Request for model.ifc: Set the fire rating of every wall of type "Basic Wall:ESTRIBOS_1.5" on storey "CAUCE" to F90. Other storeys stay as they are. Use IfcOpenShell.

First a look at what the model holds.

```python
import ifcopenshell
import ifcopenshell.util.element

model = ifcopenshell.open("model.ifc")
print(model.schema)
storey = next(s for s in model.by_type("IfcBuildingStorey") if s.Name == "CAUCE")
walls = [e for e in ifcopenshell.util.element.get_decomposition(storey) if e.is_a("IfcWall")]
seen = {}
for e in walls:
    element_type = ifcopenshell.util.element.get_type(e)
    key = (element_type.Name if element_type != e and element_type else None, ifcopenshell.util.element.get_pset(e, "Pset_WallCommon", "FireRating"))
    seen[key] = seen.get(key, 0) + 1
for (name, value), count in sorted(seen.items(), key=str):
    print(count, "x", name, "|", value)
```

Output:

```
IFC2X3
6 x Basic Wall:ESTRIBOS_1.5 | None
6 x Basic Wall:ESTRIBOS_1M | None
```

```python
import ifcopenshell
import ifcopenshell.api.pset
import ifcopenshell.util.element

model = ifcopenshell.open("model.ifc")

storey = next(s for s in model.by_type("IfcBuildingStorey") if s.Name == "CAUCE")
walls = [e for e in ifcopenshell.util.element.get_decomposition(storey) if e.is_a("IfcWall")]

count = 0
for e in walls:
    element_type = ifcopenshell.util.element.get_type(e)
    if element_type in (None, e) or element_type.Name != "Basic Wall:ESTRIBOS_1.5":
        continue
    # add_pset returns the element's existing set when there is one.
    pset = ifcopenshell.api.pset.add_pset(model, product=e, name="Pset_WallCommon")
    ifcopenshell.api.pset.edit_pset(model, pset=pset, properties={"FireRating": "F90"})
    count += 1

print(count, "walls updated")

model.write("model_v2.ifc")
```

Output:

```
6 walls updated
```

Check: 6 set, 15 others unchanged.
